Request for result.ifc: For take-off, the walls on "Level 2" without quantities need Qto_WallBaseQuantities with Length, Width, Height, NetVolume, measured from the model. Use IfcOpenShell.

First a look at what the model holds.

```python
import ifcopenshell
import ifcopenshell.util.element
import ifcopenshell.util.unit

model = ifcopenshell.open("result.ifc")
print(model.schema)
for unit_type in ("LENGTHUNIT", "AREAUNIT", "VOLUMEUNIT"):
    print(unit_type, ifcopenshell.util.unit.calculate_unit_scale(model, unit_type))
storey = next(s for s in model.by_type("IfcBuildingStorey") if s.Name == "Level 2")
walls = [e for e in ifcopenshell.util.element.get_decomposition(storey) if e.is_a("IfcWall")]
for e in sorted(walls, key=lambda e: e.id()):
    print(e.id(), e.is_a(), e.Name, list(ifcopenshell.util.element.get_psets(e, qtos_only=True)), sep=" | ")
```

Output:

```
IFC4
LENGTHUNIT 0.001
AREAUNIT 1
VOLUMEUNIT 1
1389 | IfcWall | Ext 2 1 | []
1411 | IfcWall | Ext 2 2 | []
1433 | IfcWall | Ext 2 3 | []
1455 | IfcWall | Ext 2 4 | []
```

```python
import ifcopenshell
import ifcopenshell.api.pset
import ifcopenshell.geom
import ifcopenshell.util.element
import ifcopenshell.util.shape
import ifcopenshell.util.unit

model = ifcopenshell.open("result.ifc")
unit_scale = ifcopenshell.util.unit.calculate_unit_scale(model)
volume_scale = ifcopenshell.util.unit.calculate_unit_scale(model, "VOLUMEUNIT")
settings = ifcopenshell.geom.settings()

storey = next(s for s in model.by_type("IfcBuildingStorey") if s.Name == "Level 2")
walls = [e for e in ifcopenshell.util.element.get_decomposition(storey) if e.is_a("IfcWall")]

for e in sorted(walls, key=lambda e: e.id()):
    if ifcopenshell.util.element.get_psets(e, qtos_only=True, should_inherit=False):
        continue
    # Geometry comes back in metres, in the element's own axes.
    shape = ifcopenshell.geom.create_shape(settings, e)
    values = {
        "Length": ifcopenshell.util.shape.get_x(shape.geometry) / unit_scale,
        "Width": ifcopenshell.util.shape.get_y(shape.geometry) / unit_scale,
        "Height": ifcopenshell.util.shape.get_z(shape.geometry) / unit_scale,
        "NetVolume": ifcopenshell.util.shape.get_volume(shape.geometry) / volume_scale,
    }
    qto = ifcopenshell.api.pset.add_qto(model, product=e, name="Qto_WallBaseQuantities")
    ifcopenshell.api.pset.edit_qto(model, qto=qto, properties=values)
    print(e.id(), {k: round(v, 3) for k, v in values.items()})

model.write("result_updated.ifc")
```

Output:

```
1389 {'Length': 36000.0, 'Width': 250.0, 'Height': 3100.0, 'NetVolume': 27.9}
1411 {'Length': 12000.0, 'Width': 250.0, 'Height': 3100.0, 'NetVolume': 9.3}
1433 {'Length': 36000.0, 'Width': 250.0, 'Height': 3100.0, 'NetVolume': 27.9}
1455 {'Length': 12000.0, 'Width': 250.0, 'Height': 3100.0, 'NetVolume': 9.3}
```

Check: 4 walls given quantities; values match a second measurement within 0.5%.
